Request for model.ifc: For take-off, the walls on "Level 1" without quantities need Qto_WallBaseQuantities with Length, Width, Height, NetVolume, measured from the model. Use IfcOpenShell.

First a look at what the model holds.

```python
import ifcopenshell
import ifcopenshell.util.element
import ifcopenshell.util.unit

model = ifcopenshell.open("model.ifc")
print(model.schema)
for unit_type in ("LENGTHUNIT", "AREAUNIT", "VOLUMEUNIT"):
    print(unit_type, ifcopenshell.util.unit.calculate_unit_scale(model, unit_type))
storey = next(s for s in model.by_type("IfcBuildingStorey") if s.Name == "Level 1")
walls = [e for e in ifcopenshell.util.element.get_decomposition(storey) if e.is_a("IfcWall")]
for e in sorted(walls, key=lambda e: e.id()):
    print(e.id(), e.is_a(), e.Name, list(ifcopenshell.util.element.get_psets(e, qtos_only=True)), sep=" | ")
```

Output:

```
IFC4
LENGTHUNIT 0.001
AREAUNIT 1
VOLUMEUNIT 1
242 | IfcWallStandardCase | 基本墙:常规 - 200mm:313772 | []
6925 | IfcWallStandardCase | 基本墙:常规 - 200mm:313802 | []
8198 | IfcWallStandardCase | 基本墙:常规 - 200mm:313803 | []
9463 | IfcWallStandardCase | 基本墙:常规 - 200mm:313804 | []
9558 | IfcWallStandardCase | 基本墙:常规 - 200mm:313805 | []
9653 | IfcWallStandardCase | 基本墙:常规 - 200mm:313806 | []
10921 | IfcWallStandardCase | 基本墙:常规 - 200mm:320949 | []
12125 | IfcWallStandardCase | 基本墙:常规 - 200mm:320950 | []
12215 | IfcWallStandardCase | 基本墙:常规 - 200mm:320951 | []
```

```python
import ifcopenshell
import ifcopenshell.api.pset
import ifcopenshell.geom
import ifcopenshell.util.element
import ifcopenshell.util.shape
import ifcopenshell.util.unit

model = ifcopenshell.open("model.ifc")
unit_scale = ifcopenshell.util.unit.calculate_unit_scale(model)
volume_scale = ifcopenshell.util.unit.calculate_unit_scale(model, "VOLUMEUNIT")
settings = ifcopenshell.geom.settings()

storey = next(s for s in model.by_type("IfcBuildingStorey") if s.Name == "Level 1")
walls = [e for e in ifcopenshell.util.element.get_decomposition(storey) if e.is_a("IfcWall")]

for e in sorted(walls, key=lambda e: e.id()):
    if ifcopenshell.util.element.get_psets(e, qtos_only=True, should_inherit=False):
        continue
    # Geometry comes back in metres, in the element's own axes.
    shape = ifcopenshell.geom.create_shape(settings, e)
    values = {
        "Length": ifcopenshell.util.shape.get_x(shape.geometry) / unit_scale,
        "Width": ifcopenshell.util.shape.get_y(shape.geometry) / unit_scale,
        "Height": ifcopenshell.util.shape.get_z(shape.geometry) / unit_scale,
        "NetVolume": ifcopenshell.util.shape.get_volume(shape.geometry) / volume_scale,
    }
    qto = ifcopenshell.api.pset.add_qto(model, product=e, name="Qto_WallBaseQuantities")
    ifcopenshell.api.pset.edit_qto(model, qto=qto, properties=values)
    print(e.id(), {k: round(v, 3) for k, v in values.items()})

model.write("model_rev.ifc")
```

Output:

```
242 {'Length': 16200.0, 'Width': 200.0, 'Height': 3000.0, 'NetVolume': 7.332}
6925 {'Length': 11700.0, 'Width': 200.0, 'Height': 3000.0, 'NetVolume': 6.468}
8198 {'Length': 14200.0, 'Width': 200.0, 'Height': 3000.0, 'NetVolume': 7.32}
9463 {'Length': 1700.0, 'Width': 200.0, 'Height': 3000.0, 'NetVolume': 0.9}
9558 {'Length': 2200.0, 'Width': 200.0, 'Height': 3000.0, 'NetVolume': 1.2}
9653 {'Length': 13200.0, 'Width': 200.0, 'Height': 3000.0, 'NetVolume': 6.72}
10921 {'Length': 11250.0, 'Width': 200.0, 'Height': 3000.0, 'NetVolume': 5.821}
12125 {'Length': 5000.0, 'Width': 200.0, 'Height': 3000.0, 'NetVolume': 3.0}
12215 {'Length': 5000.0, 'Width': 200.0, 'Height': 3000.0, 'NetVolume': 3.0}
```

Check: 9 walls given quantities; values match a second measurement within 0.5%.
